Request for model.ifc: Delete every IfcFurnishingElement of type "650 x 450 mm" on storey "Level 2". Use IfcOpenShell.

First a look at what the model holds.

```python
import ifcopenshell
import ifcopenshell.util.element

model = ifcopenshell.open("model.ifc")
print(model.schema)
storey = next(s for s in model.by_type("IfcBuildingStorey") if s.Name == "Level 2")
furniture = [e for e in ifcopenshell.util.element.get_decomposition(storey) if e.is_a("IfcFurnishingElement")]
seen = {}
for e in furniture:
    element_type = ifcopenshell.util.element.get_type(e)
    name = element_type.Name if element_type not in (None, e) else None
    seen[name] = seen.get(name, 0) + 1
for name, count in sorted(seen.items(), key=str):
    print(count, "x", name)
```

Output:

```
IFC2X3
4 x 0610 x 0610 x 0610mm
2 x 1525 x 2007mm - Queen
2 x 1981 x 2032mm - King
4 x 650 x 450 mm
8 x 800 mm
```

```python
import ifcopenshell
import ifcopenshell.api.root
import ifcopenshell.util.element

model = ifcopenshell.open("model.ifc")

storey = next(s for s in model.by_type("IfcBuildingStorey") if s.Name == "Level 2")
furniture = [e for e in ifcopenshell.util.element.get_decomposition(storey) if e.is_a("IfcFurnishingElement")]
targets = [e for e in furniture if (t := ifcopenshell.util.element.get_type(e)) not in (None, e) and t.Name == "650 x 450 mm"]

for e in targets:
    ifcopenshell.api.root.remove_product(model, product=e)
print(len(targets), "removed")

model.write("model_updated.ifc")
```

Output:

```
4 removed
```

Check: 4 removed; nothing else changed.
